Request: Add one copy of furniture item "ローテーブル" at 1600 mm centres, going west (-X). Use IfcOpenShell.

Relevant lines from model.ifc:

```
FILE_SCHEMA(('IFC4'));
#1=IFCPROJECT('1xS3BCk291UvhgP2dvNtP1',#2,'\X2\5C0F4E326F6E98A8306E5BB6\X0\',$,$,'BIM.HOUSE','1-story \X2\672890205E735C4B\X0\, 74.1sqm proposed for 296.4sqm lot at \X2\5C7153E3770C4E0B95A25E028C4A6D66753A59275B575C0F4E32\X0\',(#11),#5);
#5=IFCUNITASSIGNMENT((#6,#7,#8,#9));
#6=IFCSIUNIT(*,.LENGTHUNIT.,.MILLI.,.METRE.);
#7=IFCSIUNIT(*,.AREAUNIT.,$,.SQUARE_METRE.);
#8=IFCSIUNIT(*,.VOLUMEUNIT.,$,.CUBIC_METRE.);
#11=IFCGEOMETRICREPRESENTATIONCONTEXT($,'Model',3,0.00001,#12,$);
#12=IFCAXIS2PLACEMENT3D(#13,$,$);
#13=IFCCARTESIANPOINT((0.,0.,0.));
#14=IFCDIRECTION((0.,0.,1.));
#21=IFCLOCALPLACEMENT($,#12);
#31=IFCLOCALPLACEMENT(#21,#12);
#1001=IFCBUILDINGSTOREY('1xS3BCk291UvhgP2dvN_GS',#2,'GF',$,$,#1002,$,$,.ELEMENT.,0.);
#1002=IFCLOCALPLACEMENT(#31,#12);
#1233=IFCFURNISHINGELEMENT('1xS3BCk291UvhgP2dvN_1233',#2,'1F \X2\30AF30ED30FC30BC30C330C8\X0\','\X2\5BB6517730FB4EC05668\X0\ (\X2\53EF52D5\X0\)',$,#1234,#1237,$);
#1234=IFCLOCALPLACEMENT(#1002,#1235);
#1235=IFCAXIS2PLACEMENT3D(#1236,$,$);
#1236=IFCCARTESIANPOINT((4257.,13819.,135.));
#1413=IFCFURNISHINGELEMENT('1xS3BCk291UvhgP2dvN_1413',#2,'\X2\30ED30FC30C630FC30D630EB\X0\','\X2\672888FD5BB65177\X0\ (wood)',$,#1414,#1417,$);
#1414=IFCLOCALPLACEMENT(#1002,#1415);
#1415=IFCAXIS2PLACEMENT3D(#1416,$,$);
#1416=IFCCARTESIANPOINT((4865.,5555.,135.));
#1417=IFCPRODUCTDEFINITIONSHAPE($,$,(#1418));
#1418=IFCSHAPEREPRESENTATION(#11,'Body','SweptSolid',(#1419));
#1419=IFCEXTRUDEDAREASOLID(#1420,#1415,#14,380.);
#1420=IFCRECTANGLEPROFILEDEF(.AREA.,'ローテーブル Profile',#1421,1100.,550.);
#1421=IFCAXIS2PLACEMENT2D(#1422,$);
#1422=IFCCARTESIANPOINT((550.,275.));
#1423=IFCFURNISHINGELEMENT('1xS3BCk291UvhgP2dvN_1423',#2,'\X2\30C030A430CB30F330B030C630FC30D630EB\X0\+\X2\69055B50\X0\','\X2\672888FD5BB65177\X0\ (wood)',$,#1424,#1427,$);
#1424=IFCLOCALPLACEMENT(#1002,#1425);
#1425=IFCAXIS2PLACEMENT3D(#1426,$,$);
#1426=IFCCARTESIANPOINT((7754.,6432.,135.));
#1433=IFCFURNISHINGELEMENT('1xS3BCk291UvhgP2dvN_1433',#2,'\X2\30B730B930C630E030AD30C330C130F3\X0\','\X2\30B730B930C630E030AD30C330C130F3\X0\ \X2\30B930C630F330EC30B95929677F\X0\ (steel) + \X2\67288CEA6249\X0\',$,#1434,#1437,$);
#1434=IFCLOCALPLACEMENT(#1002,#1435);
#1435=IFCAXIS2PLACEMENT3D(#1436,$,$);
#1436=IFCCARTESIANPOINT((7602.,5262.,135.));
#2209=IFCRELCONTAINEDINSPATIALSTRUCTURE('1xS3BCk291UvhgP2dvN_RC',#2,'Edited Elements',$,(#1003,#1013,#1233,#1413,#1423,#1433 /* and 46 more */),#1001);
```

```python
import numpy as np
import ifcopenshell
import ifcopenshell.api.geometry
import ifcopenshell.api.root
import ifcopenshell.util.element
import ifcopenshell.util.placement

model = ifcopenshell.open("model.ifc")


def reuse_history(source, copy):
    """copy_class also copies each property set's owner history, people and application; keep the originals."""
    for rel in copy.IsDefinedBy:
        if rel.is_a("IfcRelDefinesByProperties") and (history := rel.RelatingPropertyDefinition.OwnerHistory):
            rel.RelatingPropertyDefinition.OwnerHistory = source.OwnerHistory
            ifcopenshell.util.element.remove_deep2(model, history)


source = model.by_guid("1xS3BCk291UvhgP2dvN_1413")
base = ifcopenshell.util.placement.get_local_placement(source.ObjectPlacement)
step = np.array([-1.0, 0.0, 0.0]) * 1600.0

for i in range(1, 2):
    copy = ifcopenshell.api.root.copy_class(model, product=source)
    copy.Representation = ifcopenshell.util.element.copy_deep(
        model, source.Representation, exclude=["IfcGeometricRepresentationContext", "IfcRepresentationMap"]
    )
    reuse_history(source, copy)
    matrix = base.copy()
    matrix[:3, 3] += i * step
    print("added at", matrix[:3, 3].round(3) + 0.0)
    ifcopenshell.api.geometry.edit_object_placement(model, product=copy, matrix=matrix, is_si=False)

model.write("model_v2.ifc")
```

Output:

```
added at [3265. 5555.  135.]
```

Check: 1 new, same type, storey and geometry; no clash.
